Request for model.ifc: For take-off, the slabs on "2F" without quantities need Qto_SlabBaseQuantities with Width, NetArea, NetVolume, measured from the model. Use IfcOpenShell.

First a look at what the model holds.

```python
import ifcopenshell
import ifcopenshell.util.element
import ifcopenshell.util.unit

model = ifcopenshell.open("model.ifc")
print(model.schema)
for unit_type in ("LENGTHUNIT", "AREAUNIT", "VOLUMEUNIT"):
    print(unit_type, ifcopenshell.util.unit.calculate_unit_scale(model, unit_type))
storey = next(s for s in model.by_type("IfcBuildingStorey") if s.Name == "2F")
slabs = [e for e in ifcopenshell.util.element.get_decomposition(storey) if e.is_a("IfcSlab")]
for e in sorted(slabs, key=lambda e: e.id()):
    print(e.id(), e.is_a(), e.Name, list(ifcopenshell.util.element.get_psets(e, qtos_only=True)), sep=" | ")
```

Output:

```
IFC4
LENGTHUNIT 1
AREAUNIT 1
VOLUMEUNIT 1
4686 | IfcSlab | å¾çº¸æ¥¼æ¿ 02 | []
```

```python
import ifcopenshell
import ifcopenshell.api.pset
import ifcopenshell.geom
import ifcopenshell.util.element
import ifcopenshell.util.shape
import ifcopenshell.util.unit

model = ifcopenshell.open("model.ifc")
unit_scale = ifcopenshell.util.unit.calculate_unit_scale(model)
area_scale = ifcopenshell.util.unit.calculate_unit_scale(model, "AREAUNIT")
volume_scale = ifcopenshell.util.unit.calculate_unit_scale(model, "VOLUMEUNIT")
settings = ifcopenshell.geom.settings()

storey = next(s for s in model.by_type("IfcBuildingStorey") if s.Name == "2F")
slabs = [e for e in ifcopenshell.util.element.get_decomposition(storey) if e.is_a("IfcSlab")]

for e in sorted(slabs, key=lambda e: e.id()):
    if ifcopenshell.util.element.get_psets(e, qtos_only=True, should_inherit=False):
        continue
    # Geometry comes back in metres, in the element's own axes.
    shape = ifcopenshell.geom.create_shape(settings, e)
    values = {
        "Width": ifcopenshell.util.shape.get_z(shape.geometry) / unit_scale,
        "NetArea": ifcopenshell.util.shape.get_footprint_area(shape.geometry) / area_scale,
        "NetVolume": ifcopenshell.util.shape.get_volume(shape.geometry) / volume_scale,
    }
    qto = ifcopenshell.api.pset.add_qto(model, product=e, name="Qto_SlabBaseQuantities")
    ifcopenshell.api.pset.edit_qto(model, qto=qto, properties=values)
    print(e.id(), {k: round(v, 3) for k, v in values.items()})

model.write("model_edited.ifc")
```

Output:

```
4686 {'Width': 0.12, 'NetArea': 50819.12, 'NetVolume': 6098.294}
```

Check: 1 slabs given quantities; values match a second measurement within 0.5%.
